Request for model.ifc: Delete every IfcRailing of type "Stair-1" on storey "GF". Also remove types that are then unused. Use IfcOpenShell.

First a look at what the model holds.

```python
import ifcopenshell
import ifcopenshell.util.element

model = ifcopenshell.open("model.ifc")
print(model.schema)
storey = next(s for s in model.by_type("IfcBuildingStorey") if s.Name == "GF")
railings = [e for e in ifcopenshell.util.element.get_decomposition(storey) if e.is_a("IfcRailing")]
seen = {}
for e in railings:
    element_type = ifcopenshell.util.element.get_type(e)
    name = element_type.Name if element_type not in (None, e) else None
    seen[name] = seen.get(name, 0) + 1
for name, count in sorted(seen.items(), key=str):
    print(count, "x", name)
```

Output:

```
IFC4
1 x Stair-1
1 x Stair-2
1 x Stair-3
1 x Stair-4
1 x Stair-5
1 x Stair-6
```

```python
import ifcopenshell
import ifcopenshell.api.root
import ifcopenshell.util.element

model = ifcopenshell.open("model.ifc")

storey = next(s for s in model.by_type("IfcBuildingStorey") if s.Name == "GF")
railings = [e for e in ifcopenshell.util.element.get_decomposition(storey) if e.is_a("IfcRailing")]
targets = [e for e in railings if (t := ifcopenshell.util.element.get_type(e)) not in (None, e) and t.Name == "Stair-1"]
types = {ifcopenshell.util.element.get_type(e) for e in targets} - {None, *targets}

for e in targets:
    ifcopenshell.api.root.remove_product(model, product=e)
print(len(targets), "removed")

unused = [t for t in types if not ifcopenshell.util.element.get_types(t)]
for t in unused:
    ifcopenshell.api.root.remove_product(model, product=t)
print(len(unused), "unused types removed")

model.write("model_v2.ifc")
```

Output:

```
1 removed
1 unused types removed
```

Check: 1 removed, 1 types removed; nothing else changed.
